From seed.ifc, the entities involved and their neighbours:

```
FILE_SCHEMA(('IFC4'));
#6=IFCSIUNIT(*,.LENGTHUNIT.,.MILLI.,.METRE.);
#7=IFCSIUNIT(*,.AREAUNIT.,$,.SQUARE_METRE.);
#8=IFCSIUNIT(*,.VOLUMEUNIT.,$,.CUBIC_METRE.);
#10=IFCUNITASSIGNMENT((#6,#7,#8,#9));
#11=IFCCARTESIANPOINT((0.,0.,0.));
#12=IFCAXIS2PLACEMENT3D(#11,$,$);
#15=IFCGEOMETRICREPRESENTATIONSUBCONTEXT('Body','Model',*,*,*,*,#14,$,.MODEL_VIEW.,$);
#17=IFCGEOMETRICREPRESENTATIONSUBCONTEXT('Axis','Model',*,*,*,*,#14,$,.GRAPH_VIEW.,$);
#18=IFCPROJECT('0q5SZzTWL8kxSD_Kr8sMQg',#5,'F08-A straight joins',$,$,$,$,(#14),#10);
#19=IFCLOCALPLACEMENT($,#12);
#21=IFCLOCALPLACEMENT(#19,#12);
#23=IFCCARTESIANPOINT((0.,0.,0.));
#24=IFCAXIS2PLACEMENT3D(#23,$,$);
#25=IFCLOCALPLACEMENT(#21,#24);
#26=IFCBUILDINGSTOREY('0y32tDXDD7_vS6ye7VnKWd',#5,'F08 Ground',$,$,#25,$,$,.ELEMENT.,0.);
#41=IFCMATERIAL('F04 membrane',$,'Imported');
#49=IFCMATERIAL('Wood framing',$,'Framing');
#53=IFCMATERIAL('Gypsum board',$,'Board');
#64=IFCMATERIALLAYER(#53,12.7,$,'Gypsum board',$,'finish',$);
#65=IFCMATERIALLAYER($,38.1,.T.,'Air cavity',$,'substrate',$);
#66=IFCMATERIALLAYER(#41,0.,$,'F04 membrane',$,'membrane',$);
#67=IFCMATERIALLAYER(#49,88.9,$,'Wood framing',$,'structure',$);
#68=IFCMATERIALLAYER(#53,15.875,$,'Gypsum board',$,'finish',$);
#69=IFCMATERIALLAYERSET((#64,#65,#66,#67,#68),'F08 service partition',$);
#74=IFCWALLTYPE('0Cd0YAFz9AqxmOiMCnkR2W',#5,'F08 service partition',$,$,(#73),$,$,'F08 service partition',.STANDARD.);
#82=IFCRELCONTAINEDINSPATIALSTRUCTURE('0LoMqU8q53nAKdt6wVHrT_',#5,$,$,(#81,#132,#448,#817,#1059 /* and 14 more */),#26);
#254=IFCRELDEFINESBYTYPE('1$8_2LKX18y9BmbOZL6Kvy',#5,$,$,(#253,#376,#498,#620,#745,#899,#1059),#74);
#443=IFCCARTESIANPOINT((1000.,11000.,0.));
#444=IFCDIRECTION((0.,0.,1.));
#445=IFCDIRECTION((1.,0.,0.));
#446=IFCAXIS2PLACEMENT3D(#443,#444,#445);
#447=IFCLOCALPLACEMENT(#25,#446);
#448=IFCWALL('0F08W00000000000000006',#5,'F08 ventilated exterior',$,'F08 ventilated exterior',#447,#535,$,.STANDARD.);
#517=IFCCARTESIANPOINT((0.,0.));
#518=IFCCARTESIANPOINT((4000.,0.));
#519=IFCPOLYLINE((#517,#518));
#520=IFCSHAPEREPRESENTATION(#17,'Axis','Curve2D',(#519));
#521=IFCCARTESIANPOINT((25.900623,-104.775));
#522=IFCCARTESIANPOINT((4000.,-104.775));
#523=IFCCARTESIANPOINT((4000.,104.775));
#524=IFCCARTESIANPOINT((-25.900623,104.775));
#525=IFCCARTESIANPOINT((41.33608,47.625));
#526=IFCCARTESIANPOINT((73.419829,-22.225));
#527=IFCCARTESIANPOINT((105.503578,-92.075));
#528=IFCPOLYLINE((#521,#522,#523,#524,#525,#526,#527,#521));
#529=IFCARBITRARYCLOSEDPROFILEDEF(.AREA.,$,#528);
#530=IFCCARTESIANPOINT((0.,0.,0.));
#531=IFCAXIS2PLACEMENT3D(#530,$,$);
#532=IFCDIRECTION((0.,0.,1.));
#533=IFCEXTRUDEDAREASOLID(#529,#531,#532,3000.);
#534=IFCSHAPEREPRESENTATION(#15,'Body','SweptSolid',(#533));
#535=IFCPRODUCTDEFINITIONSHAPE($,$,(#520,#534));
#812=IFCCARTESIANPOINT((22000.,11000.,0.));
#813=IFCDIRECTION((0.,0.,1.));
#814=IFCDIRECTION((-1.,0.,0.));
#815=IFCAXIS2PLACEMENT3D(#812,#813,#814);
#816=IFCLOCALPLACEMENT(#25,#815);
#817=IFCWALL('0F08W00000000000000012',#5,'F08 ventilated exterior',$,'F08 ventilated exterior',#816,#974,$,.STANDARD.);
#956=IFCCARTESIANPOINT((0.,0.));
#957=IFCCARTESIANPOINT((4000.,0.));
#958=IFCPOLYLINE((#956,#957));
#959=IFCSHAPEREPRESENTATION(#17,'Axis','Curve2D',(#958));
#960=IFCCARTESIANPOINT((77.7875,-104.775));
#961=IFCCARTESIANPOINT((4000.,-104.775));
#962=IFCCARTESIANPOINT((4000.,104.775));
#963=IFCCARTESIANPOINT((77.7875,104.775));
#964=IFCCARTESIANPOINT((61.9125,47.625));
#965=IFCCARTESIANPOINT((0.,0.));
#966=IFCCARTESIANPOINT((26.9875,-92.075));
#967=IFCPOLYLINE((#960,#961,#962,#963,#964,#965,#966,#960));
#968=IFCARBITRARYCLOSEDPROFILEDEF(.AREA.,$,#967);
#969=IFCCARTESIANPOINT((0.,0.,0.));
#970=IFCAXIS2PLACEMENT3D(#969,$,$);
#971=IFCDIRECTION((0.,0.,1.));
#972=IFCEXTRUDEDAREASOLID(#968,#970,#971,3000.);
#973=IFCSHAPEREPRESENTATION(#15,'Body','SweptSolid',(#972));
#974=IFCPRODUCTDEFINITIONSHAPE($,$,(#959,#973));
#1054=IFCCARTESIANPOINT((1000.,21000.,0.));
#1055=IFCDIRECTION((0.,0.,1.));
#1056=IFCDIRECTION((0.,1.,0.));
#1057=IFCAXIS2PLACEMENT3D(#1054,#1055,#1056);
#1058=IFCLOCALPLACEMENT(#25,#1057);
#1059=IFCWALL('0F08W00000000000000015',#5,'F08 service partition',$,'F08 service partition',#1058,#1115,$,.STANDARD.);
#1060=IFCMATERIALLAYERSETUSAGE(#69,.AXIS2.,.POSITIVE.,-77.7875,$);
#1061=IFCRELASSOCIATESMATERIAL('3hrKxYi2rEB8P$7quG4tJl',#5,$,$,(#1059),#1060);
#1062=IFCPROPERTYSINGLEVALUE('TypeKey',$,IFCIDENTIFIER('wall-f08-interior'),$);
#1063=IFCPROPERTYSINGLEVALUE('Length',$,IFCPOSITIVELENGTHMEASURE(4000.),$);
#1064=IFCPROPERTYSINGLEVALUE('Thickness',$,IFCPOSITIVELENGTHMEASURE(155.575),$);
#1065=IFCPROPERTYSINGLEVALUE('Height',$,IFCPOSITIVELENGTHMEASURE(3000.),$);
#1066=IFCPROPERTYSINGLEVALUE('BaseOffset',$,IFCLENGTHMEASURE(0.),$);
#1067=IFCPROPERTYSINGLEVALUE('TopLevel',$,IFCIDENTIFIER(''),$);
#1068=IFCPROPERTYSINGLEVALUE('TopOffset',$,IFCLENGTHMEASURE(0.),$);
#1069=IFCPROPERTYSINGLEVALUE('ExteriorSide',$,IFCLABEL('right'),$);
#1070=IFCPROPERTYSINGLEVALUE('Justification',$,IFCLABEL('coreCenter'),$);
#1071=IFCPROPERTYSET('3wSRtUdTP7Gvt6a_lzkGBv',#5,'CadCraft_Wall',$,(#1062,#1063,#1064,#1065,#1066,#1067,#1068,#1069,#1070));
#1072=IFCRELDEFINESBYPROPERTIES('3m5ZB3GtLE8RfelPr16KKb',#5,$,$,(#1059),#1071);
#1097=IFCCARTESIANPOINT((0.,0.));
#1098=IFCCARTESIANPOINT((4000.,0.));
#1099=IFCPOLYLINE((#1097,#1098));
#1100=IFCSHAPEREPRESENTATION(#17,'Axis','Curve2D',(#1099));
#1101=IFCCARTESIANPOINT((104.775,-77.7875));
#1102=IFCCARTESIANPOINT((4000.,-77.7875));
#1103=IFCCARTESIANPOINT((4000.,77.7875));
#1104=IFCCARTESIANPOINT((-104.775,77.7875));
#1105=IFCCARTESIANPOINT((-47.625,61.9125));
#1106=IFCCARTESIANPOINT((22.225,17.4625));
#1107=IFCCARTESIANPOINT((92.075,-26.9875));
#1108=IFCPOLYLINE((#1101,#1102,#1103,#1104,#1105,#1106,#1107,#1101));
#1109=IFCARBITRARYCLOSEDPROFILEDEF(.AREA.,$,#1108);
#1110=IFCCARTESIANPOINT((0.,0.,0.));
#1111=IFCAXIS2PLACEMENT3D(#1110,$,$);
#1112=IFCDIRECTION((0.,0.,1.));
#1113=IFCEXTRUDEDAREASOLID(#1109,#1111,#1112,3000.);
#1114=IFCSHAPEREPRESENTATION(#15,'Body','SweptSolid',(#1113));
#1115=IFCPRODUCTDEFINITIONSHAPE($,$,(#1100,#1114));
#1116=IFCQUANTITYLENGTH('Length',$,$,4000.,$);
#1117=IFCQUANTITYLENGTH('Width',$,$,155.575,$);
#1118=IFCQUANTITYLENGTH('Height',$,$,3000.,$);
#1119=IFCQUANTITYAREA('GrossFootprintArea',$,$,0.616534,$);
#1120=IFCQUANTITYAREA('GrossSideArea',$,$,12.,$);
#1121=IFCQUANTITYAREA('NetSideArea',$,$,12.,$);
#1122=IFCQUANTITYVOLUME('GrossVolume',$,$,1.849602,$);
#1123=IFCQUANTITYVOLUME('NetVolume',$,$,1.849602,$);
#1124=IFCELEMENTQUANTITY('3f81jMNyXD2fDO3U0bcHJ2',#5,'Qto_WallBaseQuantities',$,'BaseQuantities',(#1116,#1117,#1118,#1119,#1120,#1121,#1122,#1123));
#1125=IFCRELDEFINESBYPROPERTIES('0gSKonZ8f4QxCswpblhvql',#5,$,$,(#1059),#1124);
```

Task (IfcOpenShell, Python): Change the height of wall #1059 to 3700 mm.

```python
import ifcopenshell
import ifcopenshell.api.pset
import ifcopenshell.geom
import ifcopenshell.util.element
import ifcopenshell.util.representation
import ifcopenshell.util.shape
import ifcopenshell.util.unit

model = ifcopenshell.open("seed.ifc")
unit_scale = ifcopenshell.util.unit.calculate_unit_scale(model)
area_scale = ifcopenshell.util.unit.calculate_unit_scale(model, "AREAUNIT")
volume_scale = ifcopenshell.util.unit.calculate_unit_scale(model, "VOLUMEUNIT")
settings = ifcopenshell.geom.settings()


def volume(element):
    """Net volume in cubic metres, openings subtracted."""
    shape = ifcopenshell.geom.create_shape(settings, element)
    return ifcopenshell.util.shape.get_volume(shape.geometry)


wall = model.by_id(1059)
before = volume(wall)

body = ifcopenshell.util.representation.get_representation(wall, "Model", "Body")
solid = body.Items[0]
old_height = solid.Depth
solid.Depth = 3.7 / unit_scale
after = volume(wall)
thickness = 0.1556  # wall thickness in metres

# Update the stored height, areas and volumes.
pset = model.by_id(ifcopenshell.util.element.get_pset(wall, "CadCraft_Wall", should_inherit=False)["id"])
ifcopenshell.api.pset.edit_pset(model, pset=pset, properties={
    "Height": model.create_entity("IfcPositiveLengthMeasure", solid.Depth),
})
qto = model.by_id(ifcopenshell.util.element.get_pset(wall, "Qto_WallBaseQuantities", should_inherit=False)["id"])
ifcopenshell.api.pset.edit_qto(model, qto=qto, properties={
    "Height": solid.Depth,
    "GrossSideArea": ifcopenshell.util.element.get_pset(wall, "Qto_WallBaseQuantities", "GrossSideArea") * solid.Depth / old_height,
    "NetSideArea": after / thickness / area_scale,
    "GrossVolume": ifcopenshell.util.element.get_pset(wall, "Qto_WallBaseQuantities", "GrossVolume") * solid.Depth / old_height,
    "NetVolume": after / volume_scale,
})

print(f"height {old_height:g} -> {solid.Depth:g}, volume {before:.3f} -> {after:.3f} m3")

model.write("seed-out.ifc")
```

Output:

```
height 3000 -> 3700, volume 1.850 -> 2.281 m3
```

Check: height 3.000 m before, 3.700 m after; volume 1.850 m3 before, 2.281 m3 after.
